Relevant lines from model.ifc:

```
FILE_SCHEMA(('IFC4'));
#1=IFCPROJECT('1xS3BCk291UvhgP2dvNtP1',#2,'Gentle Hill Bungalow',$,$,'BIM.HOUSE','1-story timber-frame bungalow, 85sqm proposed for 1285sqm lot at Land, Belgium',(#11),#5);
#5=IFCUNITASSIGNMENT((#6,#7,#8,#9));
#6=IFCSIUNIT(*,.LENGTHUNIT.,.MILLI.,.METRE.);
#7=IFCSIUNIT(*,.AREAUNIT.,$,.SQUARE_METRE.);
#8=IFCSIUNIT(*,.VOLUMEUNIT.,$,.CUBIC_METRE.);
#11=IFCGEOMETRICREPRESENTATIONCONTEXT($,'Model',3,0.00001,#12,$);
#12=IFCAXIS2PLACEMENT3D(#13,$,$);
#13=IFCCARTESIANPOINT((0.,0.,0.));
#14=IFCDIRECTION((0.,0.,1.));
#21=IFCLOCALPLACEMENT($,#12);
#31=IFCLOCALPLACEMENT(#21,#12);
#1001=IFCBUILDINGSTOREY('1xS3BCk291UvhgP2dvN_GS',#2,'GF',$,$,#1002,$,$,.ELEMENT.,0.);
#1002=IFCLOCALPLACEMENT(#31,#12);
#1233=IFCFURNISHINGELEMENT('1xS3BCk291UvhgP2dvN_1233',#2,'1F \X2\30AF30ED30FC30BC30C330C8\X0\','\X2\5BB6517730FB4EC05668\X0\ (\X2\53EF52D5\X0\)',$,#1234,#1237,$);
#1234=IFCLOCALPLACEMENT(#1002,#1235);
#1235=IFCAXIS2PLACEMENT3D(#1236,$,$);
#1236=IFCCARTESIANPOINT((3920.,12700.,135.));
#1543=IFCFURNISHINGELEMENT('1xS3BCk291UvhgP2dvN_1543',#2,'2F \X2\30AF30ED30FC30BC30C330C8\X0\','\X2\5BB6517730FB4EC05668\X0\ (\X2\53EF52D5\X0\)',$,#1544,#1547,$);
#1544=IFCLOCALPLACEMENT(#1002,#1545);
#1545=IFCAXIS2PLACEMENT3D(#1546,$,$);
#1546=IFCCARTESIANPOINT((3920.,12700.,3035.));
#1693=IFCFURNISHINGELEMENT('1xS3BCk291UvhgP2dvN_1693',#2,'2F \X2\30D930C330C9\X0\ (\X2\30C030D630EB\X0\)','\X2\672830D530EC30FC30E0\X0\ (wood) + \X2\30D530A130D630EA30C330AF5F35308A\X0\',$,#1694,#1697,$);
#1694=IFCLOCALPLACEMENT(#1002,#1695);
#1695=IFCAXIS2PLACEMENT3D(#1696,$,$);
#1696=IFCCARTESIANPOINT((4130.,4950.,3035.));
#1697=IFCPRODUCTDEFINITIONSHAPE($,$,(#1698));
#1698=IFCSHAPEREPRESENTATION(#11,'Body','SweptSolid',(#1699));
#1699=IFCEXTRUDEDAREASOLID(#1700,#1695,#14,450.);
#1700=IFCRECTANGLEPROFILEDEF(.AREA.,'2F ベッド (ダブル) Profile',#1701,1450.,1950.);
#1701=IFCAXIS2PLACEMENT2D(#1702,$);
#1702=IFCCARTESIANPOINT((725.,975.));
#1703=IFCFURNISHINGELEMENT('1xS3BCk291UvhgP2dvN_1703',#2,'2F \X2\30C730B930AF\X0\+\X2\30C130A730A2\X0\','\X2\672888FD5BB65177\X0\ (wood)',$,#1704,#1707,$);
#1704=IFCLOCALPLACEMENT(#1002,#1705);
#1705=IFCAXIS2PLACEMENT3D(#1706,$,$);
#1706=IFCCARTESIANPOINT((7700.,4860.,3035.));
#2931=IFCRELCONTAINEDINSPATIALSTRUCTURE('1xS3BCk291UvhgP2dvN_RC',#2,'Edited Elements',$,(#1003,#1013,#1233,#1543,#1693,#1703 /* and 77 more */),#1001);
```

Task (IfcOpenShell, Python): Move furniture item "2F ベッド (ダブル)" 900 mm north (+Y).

```python
import ifcopenshell
import ifcopenshell.api.geometry
import ifcopenshell.util.placement
import ifcopenshell.util.unit

model = ifcopenshell.open("model.ifc")
unit_scale = ifcopenshell.util.unit.calculate_unit_scale(model)

item = model.by_guid("1xS3BCk291UvhgP2dvN_1693")
matrix = ifcopenshell.util.placement.get_local_placement(item.ObjectPlacement)
matrix[1, 3] += 0.9 / unit_scale
ifcopenshell.api.geometry.edit_object_placement(model, product=item, matrix=matrix, is_si=False)

print(ifcopenshell.util.placement.get_local_placement(item.ObjectPlacement).round(3) + 0.0)

model.write("model_v2.ifc")
```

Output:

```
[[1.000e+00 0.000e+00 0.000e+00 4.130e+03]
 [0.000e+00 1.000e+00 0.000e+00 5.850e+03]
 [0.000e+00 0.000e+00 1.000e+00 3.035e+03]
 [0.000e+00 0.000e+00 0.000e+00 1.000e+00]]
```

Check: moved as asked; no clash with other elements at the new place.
